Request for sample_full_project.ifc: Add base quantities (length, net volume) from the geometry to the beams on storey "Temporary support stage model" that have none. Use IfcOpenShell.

First a look at what the model holds.

```python
import ifcopenshell
import ifcopenshell.util.element
import ifcopenshell.util.unit

model = ifcopenshell.open("sample_full_project.ifc")
print(model.schema)
for unit_type in ("LENGTHUNIT", "AREAUNIT", "VOLUMEUNIT"):
    print(unit_type, ifcopenshell.util.unit.calculate_unit_scale(model, unit_type))
storey = next(s for s in model.by_type("IfcBuildingStorey") if s.Name == "Temporary support stage model")
beams = [e for e in ifcopenshell.util.element.get_decomposition(storey) if e.is_a("IfcBeam")]
for e in sorted(beams, key=lambda e: e.id()):
    print(e.id(), e.is_a(), e.Name, list(ifcopenshell.util.element.get_psets(e, qtos_only=True)), sep=" | ")
```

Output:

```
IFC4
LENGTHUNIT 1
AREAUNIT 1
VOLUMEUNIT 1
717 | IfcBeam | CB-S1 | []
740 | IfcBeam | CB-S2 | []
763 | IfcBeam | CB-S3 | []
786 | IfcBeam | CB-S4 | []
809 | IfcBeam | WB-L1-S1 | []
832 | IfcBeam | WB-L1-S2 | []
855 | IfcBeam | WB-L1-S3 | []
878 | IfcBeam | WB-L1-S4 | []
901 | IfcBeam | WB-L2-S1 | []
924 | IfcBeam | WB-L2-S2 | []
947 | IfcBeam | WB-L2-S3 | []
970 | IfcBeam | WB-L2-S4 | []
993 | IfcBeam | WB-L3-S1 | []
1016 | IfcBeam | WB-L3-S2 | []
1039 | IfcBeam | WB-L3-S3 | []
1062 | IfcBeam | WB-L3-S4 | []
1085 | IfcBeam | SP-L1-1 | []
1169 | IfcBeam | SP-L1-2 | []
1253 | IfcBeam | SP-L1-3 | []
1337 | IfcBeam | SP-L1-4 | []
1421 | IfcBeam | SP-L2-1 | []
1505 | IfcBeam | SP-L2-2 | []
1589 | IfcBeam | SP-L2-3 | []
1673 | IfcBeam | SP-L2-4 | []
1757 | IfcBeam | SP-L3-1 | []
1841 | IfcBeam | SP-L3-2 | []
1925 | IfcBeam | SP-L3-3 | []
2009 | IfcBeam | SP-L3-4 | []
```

```python
import ifcopenshell
import ifcopenshell.api.pset
import ifcopenshell.geom
import ifcopenshell.util.element
import ifcopenshell.util.shape
import ifcopenshell.util.unit

model = ifcopenshell.open("sample_full_project.ifc")
unit_scale = ifcopenshell.util.unit.calculate_unit_scale(model)
volume_scale = ifcopenshell.util.unit.calculate_unit_scale(model, "VOLUMEUNIT")
settings = ifcopenshell.geom.settings()

storey = next(s for s in model.by_type("IfcBuildingStorey") if s.Name == "Temporary support stage model")
beams = [e for e in ifcopenshell.util.element.get_decomposition(storey) if e.is_a("IfcBeam")]

for e in sorted(beams, key=lambda e: e.id()):
    if ifcopenshell.util.element.get_psets(e, qtos_only=True, should_inherit=False):
        continue
    # Geometry comes back in metres, in the element's own axes.
    shape = ifcopenshell.geom.create_shape(settings, e)
    values = {
        "Length": ifcopenshell.util.shape.get_max_xyz(shape.geometry) / unit_scale,
        "NetVolume": ifcopenshell.util.shape.get_volume(shape.geometry) / volume_scale,
    }
    qto = ifcopenshell.api.pset.add_qto(model, product=e, name="Qto_BeamBaseQuantities")
    ifcopenshell.api.pset.edit_qto(model, qto=qto, properties=values)
    print(e.id(), {k: round(v, 3) for k, v in values.items()})

model.write("sample_full_project_updated.ifc")
```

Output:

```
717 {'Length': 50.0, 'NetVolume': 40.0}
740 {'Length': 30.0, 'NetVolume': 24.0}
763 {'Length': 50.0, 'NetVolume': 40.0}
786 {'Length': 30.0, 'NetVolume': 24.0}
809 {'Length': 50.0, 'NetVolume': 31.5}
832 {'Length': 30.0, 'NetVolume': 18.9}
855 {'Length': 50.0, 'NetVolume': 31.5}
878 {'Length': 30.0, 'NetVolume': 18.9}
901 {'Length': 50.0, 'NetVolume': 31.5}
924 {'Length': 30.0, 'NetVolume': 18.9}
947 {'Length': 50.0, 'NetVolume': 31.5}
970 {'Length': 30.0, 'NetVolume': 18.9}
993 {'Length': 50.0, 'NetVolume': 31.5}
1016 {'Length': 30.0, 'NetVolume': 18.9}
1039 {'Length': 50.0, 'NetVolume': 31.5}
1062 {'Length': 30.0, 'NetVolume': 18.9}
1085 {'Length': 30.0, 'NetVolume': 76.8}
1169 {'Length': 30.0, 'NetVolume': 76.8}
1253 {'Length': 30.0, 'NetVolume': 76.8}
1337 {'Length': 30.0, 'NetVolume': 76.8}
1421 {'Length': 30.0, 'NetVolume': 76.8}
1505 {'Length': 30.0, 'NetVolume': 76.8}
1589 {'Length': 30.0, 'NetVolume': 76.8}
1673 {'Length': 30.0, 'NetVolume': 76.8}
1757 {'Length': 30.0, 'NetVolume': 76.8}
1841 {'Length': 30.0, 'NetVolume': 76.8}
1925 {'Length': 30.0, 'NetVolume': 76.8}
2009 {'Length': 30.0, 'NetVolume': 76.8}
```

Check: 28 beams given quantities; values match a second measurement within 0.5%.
